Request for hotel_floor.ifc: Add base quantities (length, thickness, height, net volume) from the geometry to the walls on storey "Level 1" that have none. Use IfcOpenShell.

First a look at what the model holds.

```python
import ifcopenshell
import ifcopenshell.util.element
import ifcopenshell.util.unit

model = ifcopenshell.open("hotel_floor.ifc")
print(model.schema)
for unit_type in ("LENGTHUNIT", "AREAUNIT", "VOLUMEUNIT"):
    print(unit_type, ifcopenshell.util.unit.calculate_unit_scale(model, unit_type))
storey = next(s for s in model.by_type("IfcBuildingStorey") if s.Name == "Level 1")
walls = [e for e in ifcopenshell.util.element.get_decomposition(storey) if e.is_a("IfcWall")]
for e in sorted(walls, key=lambda e: e.id()):
    print(e.id(), e.is_a(), e.Name, list(ifcopenshell.util.element.get_psets(e, qtos_only=True)), sep=" | ")
```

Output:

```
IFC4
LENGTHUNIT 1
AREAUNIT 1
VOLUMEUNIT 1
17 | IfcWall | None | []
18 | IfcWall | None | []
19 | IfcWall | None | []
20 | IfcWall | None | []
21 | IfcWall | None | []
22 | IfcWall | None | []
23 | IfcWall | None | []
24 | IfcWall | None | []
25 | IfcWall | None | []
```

```python
import ifcopenshell
import ifcopenshell.api.pset
import ifcopenshell.geom
import ifcopenshell.util.element
import ifcopenshell.util.shape
import ifcopenshell.util.unit

model = ifcopenshell.open("hotel_floor.ifc")
unit_scale = ifcopenshell.util.unit.calculate_unit_scale(model)
volume_scale = ifcopenshell.util.unit.calculate_unit_scale(model, "VOLUMEUNIT")
settings = ifcopenshell.geom.settings()

storey = next(s for s in model.by_type("IfcBuildingStorey") if s.Name == "Level 1")
walls = [e for e in ifcopenshell.util.element.get_decomposition(storey) if e.is_a("IfcWall")]

for e in sorted(walls, key=lambda e: e.id()):
    if ifcopenshell.util.element.get_psets(e, qtos_only=True, should_inherit=False):
        continue
    # Geometry comes back in metres, in the element's own axes.
    shape = ifcopenshell.geom.create_shape(settings, e)
    values = {
        "Length": ifcopenshell.util.shape.get_x(shape.geometry) / unit_scale,
        "Width": ifcopenshell.util.shape.get_y(shape.geometry) / unit_scale,
        "Height": ifcopenshell.util.shape.get_z(shape.geometry) / unit_scale,
        "NetVolume": ifcopenshell.util.shape.get_volume(shape.geometry) / volume_scale,
    }
    qto = ifcopenshell.api.pset.add_qto(model, product=e, name="Qto_WallBaseQuantities")
    ifcopenshell.api.pset.edit_qto(model, qto=qto, properties=values)
    print(e.id(), {k: round(v, 3) for k, v in values.items()})

model.write("hotel_floor_edited.ifc")
```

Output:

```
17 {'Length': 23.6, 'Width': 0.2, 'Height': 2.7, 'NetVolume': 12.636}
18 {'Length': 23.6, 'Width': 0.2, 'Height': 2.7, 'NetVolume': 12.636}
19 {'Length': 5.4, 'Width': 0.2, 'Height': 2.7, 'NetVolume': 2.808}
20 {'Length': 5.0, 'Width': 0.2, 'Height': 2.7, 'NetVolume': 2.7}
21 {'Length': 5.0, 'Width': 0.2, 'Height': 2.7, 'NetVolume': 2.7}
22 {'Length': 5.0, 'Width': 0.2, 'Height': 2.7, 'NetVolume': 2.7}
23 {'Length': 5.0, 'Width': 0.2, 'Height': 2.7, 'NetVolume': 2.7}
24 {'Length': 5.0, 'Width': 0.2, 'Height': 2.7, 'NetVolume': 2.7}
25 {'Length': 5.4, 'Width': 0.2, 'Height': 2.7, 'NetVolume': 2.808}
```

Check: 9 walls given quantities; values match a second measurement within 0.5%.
